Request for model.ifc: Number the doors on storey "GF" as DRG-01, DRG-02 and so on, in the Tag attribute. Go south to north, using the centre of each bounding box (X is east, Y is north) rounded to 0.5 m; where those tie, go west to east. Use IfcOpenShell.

First a look at what the model holds.

```python
import ifcopenshell
import ifcopenshell.util.element
import ifcopenshell.util.placement

model = ifcopenshell.open("model.ifc")
print(model.schema)
storey = next(s for s in model.by_type("IfcBuildingStorey") if s.Name == "GF")
doors = [e for e in ifcopenshell.util.element.get_decomposition(storey) if e.is_a("IfcDoor")]
for e in sorted(doors, key=lambda e: e.id()):
    origin = ifcopenshell.util.placement.get_local_placement(e.ObjectPlacement)[:3, 3]
    print(e.id(), e.Tag, e.Name, origin.round(2) + 0.0, sep=" | ")
```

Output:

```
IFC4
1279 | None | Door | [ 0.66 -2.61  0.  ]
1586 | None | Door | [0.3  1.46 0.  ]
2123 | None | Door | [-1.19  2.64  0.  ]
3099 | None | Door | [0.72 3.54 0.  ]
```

```python
import ifcopenshell
import ifcopenshell.geom
import ifcopenshell.util.element
import ifcopenshell.util.shape

model = ifcopenshell.open("model.ifc")
settings = ifcopenshell.geom.settings()
settings.set("use-world-coords", True)


def centre(element):
    shape = ifcopenshell.geom.create_shape(settings, element)
    return ifcopenshell.util.shape.get_bbox_centroid(shape.geometry)


storey = next(s for s in model.by_type("IfcBuildingStorey") if s.Name == "GF")
doors = [e for e in ifcopenshell.util.element.get_decomposition(storey) if e.is_a("IfcDoor")]

# Insertion points can sit at a corner or the storey origin, so sort by the geometry (in metres).
centres = {e: centre(e) for e in doors}
doors.sort(key=lambda e: (round(centres[e][1] / 0.5), centres[e][0]))

for i, e in enumerate(doors, start=1):
    number = f"DRG-{i:02d}"
    e.Tag = number
    print(e.id(), number)

model.write("model-out.ifc")
```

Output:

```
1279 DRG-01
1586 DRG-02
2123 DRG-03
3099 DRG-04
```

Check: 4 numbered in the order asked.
